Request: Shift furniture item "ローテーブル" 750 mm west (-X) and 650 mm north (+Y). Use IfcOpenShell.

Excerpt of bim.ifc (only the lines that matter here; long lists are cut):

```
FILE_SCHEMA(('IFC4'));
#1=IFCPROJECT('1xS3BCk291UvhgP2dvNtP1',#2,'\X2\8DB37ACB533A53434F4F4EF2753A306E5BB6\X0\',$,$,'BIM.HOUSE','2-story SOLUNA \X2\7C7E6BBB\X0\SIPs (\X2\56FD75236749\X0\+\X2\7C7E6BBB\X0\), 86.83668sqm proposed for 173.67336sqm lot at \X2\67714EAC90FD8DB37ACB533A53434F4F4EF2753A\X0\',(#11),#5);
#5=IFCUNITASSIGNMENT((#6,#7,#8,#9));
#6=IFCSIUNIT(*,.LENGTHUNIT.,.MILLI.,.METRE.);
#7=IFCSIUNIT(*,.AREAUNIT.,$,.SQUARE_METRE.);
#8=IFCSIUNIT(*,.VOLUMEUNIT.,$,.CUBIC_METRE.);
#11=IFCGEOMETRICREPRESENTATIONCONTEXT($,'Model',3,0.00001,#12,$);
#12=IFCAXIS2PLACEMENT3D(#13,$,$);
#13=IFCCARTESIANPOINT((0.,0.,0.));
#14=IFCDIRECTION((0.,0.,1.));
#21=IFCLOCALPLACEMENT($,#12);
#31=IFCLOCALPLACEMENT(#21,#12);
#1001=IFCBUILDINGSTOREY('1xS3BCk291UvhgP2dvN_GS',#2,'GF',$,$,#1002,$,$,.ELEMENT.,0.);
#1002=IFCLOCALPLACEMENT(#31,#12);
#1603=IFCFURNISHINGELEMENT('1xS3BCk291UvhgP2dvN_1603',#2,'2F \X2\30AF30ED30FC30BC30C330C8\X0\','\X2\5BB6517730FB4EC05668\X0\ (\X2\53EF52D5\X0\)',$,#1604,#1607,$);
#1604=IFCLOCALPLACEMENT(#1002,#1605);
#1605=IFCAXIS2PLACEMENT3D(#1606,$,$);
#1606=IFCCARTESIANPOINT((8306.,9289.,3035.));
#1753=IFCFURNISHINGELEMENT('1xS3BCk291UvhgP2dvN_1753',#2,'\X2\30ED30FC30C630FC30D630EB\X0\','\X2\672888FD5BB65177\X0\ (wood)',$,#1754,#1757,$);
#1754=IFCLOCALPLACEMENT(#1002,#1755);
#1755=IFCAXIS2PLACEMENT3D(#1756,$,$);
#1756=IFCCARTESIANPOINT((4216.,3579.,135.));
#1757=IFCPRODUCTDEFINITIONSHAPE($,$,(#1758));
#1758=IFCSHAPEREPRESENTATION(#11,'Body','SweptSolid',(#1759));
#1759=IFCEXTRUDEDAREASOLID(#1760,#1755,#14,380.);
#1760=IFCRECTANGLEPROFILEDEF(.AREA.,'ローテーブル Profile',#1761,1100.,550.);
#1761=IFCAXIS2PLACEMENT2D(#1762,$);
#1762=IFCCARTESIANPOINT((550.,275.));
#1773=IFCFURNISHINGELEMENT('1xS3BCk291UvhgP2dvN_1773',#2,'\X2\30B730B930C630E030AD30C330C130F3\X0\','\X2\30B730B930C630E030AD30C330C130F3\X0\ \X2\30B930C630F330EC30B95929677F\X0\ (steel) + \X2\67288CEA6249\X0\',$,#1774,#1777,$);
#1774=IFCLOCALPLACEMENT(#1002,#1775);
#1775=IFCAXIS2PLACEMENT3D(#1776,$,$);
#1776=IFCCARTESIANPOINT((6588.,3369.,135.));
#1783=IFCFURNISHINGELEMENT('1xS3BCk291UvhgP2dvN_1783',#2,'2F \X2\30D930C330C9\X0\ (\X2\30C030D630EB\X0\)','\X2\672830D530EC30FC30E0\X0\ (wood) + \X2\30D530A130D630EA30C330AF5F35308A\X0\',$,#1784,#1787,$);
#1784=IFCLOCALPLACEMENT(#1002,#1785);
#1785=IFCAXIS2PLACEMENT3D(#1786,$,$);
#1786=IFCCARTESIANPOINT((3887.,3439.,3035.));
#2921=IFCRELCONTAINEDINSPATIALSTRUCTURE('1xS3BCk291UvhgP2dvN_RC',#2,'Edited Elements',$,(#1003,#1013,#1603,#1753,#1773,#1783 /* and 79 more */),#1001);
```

```python
import ifcopenshell
import ifcopenshell.api.geometry
import ifcopenshell.util.placement

model = ifcopenshell.open("bim.ifc")

item = model.by_guid("1xS3BCk291UvhgP2dvN_1753")
matrix = ifcopenshell.util.placement.get_local_placement(item.ObjectPlacement)
matrix[0, 3] -= 750.0
matrix[1, 3] += 650.0
ifcopenshell.api.geometry.edit_object_placement(model, product=item, matrix=matrix, is_si=False)

print(ifcopenshell.util.placement.get_local_placement(item.ObjectPlacement).round(3) + 0.0)

model.write("bim_updated.ifc")
```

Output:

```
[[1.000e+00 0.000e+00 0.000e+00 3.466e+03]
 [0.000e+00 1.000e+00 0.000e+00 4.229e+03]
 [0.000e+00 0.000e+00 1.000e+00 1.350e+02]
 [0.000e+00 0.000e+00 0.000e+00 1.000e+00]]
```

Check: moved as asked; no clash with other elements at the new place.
